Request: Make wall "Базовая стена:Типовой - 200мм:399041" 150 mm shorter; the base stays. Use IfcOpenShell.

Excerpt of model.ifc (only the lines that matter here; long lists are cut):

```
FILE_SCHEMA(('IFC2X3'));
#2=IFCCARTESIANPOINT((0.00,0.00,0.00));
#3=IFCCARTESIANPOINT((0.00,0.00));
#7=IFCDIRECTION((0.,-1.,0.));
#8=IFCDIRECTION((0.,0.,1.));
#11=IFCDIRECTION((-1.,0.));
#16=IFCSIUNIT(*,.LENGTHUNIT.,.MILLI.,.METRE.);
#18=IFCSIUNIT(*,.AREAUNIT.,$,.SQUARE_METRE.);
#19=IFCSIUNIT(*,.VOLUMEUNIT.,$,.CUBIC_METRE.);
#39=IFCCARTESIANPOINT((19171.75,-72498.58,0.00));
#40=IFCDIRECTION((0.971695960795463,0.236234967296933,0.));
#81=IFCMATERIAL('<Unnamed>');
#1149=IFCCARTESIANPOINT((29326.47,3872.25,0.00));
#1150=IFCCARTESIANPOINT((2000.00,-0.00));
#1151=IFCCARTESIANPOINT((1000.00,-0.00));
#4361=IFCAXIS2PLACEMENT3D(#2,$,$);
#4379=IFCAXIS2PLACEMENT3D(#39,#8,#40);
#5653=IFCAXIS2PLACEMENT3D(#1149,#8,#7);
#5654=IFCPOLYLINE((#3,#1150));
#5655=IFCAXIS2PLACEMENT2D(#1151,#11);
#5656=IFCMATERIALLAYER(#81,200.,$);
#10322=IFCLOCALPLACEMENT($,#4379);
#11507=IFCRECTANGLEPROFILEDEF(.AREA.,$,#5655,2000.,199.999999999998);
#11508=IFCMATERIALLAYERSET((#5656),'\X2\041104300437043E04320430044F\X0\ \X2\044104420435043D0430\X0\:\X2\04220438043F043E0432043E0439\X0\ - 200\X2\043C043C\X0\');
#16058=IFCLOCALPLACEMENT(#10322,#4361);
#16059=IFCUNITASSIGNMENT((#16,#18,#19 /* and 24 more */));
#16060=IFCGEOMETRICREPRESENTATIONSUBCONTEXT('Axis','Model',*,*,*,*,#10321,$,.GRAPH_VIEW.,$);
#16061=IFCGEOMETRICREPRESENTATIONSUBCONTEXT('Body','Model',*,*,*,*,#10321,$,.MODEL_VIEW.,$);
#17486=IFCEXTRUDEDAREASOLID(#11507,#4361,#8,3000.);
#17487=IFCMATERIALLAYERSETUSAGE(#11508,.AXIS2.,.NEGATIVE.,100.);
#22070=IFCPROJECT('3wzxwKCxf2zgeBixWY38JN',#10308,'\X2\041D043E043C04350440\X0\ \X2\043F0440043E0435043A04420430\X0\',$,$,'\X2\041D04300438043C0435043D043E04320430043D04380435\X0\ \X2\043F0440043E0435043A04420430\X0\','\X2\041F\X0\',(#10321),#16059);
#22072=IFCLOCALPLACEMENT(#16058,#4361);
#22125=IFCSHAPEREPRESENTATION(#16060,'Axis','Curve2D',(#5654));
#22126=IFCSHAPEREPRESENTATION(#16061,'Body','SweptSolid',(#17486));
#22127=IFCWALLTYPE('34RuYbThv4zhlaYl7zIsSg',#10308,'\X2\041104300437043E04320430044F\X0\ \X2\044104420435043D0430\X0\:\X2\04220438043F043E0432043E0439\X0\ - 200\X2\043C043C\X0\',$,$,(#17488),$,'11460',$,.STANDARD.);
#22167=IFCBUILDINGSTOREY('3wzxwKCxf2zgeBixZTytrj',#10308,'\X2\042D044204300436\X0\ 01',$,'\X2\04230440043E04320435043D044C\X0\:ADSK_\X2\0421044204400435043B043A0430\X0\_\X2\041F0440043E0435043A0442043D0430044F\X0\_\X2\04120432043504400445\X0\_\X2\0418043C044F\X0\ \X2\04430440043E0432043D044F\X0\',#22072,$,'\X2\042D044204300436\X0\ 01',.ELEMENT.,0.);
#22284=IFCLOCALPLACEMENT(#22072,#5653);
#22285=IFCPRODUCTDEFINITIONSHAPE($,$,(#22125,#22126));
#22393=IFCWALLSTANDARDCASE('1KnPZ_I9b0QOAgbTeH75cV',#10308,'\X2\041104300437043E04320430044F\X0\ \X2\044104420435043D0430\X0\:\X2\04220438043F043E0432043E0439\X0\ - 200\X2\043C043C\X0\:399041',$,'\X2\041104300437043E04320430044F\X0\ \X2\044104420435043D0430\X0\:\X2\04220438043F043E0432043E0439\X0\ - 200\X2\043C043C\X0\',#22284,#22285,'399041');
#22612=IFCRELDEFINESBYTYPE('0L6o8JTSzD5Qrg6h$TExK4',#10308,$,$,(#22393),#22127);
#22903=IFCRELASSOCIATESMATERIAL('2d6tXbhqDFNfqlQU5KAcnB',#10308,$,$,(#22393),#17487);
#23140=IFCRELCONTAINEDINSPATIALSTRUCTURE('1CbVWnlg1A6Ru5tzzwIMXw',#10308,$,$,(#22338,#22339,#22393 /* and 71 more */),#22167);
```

```python
import ifcopenshell
import ifcopenshell.geom
import ifcopenshell.util.representation
import ifcopenshell.util.shape
import ifcopenshell.util.unit

model = ifcopenshell.open("model.ifc")
unit_scale = ifcopenshell.util.unit.calculate_unit_scale(model)
settings = ifcopenshell.geom.settings()


def volume(element):
    """Net volume in cubic metres, openings subtracted."""
    shape = ifcopenshell.geom.create_shape(settings, element)
    return ifcopenshell.util.shape.get_volume(shape.geometry)


wall = model.by_guid("1KnPZ_I9b0QOAgbTeH75cV")
before = volume(wall)

body = ifcopenshell.util.representation.get_representation(wall, "Model", "Body")
solid = body.Items[0]
old_height = solid.Depth
solid.Depth -= 0.15 / unit_scale
after = volume(wall)

print(f"height {old_height:g} -> {solid.Depth:g}, volume {before:.3f} -> {after:.3f} m3")

model.write("model-out.ifc")
```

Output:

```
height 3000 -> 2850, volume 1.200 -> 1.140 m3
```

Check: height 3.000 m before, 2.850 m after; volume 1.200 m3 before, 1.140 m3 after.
